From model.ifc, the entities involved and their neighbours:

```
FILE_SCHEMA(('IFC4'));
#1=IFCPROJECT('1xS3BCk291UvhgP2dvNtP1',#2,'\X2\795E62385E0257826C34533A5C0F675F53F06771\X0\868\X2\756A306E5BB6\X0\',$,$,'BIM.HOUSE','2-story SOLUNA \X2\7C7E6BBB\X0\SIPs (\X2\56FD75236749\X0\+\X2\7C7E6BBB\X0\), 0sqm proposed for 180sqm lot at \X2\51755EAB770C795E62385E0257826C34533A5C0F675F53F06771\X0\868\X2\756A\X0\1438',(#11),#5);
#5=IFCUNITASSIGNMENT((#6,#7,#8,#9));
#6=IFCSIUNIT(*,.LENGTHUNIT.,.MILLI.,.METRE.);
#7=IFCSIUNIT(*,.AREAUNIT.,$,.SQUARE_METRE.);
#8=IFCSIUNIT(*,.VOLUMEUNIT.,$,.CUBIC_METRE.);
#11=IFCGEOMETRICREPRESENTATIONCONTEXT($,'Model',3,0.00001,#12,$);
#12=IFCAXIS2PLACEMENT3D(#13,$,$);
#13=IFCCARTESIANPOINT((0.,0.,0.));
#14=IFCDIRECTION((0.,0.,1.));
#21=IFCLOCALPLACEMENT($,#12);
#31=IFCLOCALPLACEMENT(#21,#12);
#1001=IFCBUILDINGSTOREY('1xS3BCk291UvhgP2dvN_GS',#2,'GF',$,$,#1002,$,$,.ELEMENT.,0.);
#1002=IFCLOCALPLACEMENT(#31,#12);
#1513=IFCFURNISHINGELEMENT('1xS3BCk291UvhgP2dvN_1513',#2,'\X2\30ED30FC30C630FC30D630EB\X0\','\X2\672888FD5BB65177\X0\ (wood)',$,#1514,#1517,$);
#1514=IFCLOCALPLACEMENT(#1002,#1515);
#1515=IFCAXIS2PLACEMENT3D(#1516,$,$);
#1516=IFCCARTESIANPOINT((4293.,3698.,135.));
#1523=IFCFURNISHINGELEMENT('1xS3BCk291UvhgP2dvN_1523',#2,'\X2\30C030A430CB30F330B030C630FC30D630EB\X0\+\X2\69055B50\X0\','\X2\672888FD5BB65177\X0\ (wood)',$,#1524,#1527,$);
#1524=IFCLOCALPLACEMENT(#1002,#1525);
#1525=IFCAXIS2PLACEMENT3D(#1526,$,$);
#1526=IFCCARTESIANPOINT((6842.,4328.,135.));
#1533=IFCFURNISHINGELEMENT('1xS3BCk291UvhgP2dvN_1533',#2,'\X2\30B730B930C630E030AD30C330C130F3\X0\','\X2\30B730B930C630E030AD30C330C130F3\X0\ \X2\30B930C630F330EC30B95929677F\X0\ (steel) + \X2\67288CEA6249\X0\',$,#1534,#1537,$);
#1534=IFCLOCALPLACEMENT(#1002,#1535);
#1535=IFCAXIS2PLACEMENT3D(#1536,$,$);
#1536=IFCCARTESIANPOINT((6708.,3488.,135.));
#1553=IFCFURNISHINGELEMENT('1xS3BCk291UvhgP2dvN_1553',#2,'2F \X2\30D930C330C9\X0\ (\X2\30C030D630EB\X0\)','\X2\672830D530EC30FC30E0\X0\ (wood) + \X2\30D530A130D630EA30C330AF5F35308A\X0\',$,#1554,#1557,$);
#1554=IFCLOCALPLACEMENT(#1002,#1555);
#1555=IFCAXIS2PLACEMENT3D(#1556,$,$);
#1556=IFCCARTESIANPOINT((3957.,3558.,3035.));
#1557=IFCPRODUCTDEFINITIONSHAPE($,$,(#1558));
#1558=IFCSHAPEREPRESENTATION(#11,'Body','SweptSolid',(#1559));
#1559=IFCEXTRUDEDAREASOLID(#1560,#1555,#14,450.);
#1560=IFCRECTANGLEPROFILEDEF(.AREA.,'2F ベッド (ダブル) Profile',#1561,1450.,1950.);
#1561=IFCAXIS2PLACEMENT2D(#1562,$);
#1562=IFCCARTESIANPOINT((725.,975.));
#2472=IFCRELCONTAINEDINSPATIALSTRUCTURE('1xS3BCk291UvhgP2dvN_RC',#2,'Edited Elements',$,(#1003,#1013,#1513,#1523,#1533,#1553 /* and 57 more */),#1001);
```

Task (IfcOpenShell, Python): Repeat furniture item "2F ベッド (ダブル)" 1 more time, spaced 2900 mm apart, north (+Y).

```python
import numpy as np
import ifcopenshell
import ifcopenshell.api.geometry
import ifcopenshell.api.root
import ifcopenshell.util.element
import ifcopenshell.util.placement
import ifcopenshell.util.unit

model = ifcopenshell.open("model.ifc")
unit_scale = ifcopenshell.util.unit.calculate_unit_scale(model)


def reuse_history(source, copy):
    """copy_class also copies each property set's owner history, people and application; keep the originals."""
    for rel in copy.IsDefinedBy:
        if rel.is_a("IfcRelDefinesByProperties") and (history := rel.RelatingPropertyDefinition.OwnerHistory):
            rel.RelatingPropertyDefinition.OwnerHistory = source.OwnerHistory
            ifcopenshell.util.element.remove_deep2(model, history)


source = model.by_guid("1xS3BCk291UvhgP2dvN_1553")
base = ifcopenshell.util.placement.get_local_placement(source.ObjectPlacement)
step = np.array([0.0, 1.0, 0.0]) * 2.9 / unit_scale

for i in range(1, 2):
    copy = ifcopenshell.api.root.copy_class(model, product=source)
    copy.Representation = ifcopenshell.util.element.copy_deep(
        model, source.Representation, exclude=["IfcGeometricRepresentationContext", "IfcRepresentationMap"]
    )
    reuse_history(source, copy)
    matrix = base.copy()
    matrix[:3, 3] += i * step
    print("added at", matrix[:3, 3].round(3) + 0.0)
    ifcopenshell.api.geometry.edit_object_placement(model, product=copy, matrix=matrix, is_si=False)

model.write("model-out.ifc")
```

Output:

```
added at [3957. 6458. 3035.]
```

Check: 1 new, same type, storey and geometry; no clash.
